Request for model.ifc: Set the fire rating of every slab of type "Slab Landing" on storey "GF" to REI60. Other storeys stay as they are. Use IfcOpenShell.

First a look at what the model holds.

```python
import ifcopenshell
import ifcopenshell.util.element

model = ifcopenshell.open("model.ifc")
print(model.schema)
storey = next(s for s in model.by_type("IfcBuildingStorey") if s.Name == "GF")
slabs = [e for e in ifcopenshell.util.element.get_decomposition(storey) if e.is_a("IfcSlab")]
seen = {}
for e in slabs:
    element_type = ifcopenshell.util.element.get_type(e)
    key = (element_type.Name if element_type != e and element_type else None, ifcopenshell.util.element.get_pset(e, "Pset_SlabCommon", "FireRating"))
    seen[key] = seen.get(key, 0) + 1
for (name, value), count in sorted(seen.items(), key=str):
    print(count, "x", name, "|", value)
```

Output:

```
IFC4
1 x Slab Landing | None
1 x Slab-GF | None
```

```python
import ifcopenshell
import ifcopenshell.api.pset
import ifcopenshell.util.element

model = ifcopenshell.open("model.ifc")

storey = next(s for s in model.by_type("IfcBuildingStorey") if s.Name == "GF")
slabs = [e for e in ifcopenshell.util.element.get_decomposition(storey) if e.is_a("IfcSlab")]

count = 0
for e in slabs:
    element_type = ifcopenshell.util.element.get_type(e)
    if element_type in (None, e) or element_type.Name != "Slab Landing":
        continue
    # add_pset returns the element's existing set when there is one.
    pset = ifcopenshell.api.pset.add_pset(model, product=e, name="Pset_SlabCommon")
    ifcopenshell.api.pset.edit_pset(model, pset=pset, properties={"FireRating": "REI60"})
    count += 1

print(count, "slabs updated")

model.write("model_v2.ifc")
```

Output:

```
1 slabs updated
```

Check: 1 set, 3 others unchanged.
